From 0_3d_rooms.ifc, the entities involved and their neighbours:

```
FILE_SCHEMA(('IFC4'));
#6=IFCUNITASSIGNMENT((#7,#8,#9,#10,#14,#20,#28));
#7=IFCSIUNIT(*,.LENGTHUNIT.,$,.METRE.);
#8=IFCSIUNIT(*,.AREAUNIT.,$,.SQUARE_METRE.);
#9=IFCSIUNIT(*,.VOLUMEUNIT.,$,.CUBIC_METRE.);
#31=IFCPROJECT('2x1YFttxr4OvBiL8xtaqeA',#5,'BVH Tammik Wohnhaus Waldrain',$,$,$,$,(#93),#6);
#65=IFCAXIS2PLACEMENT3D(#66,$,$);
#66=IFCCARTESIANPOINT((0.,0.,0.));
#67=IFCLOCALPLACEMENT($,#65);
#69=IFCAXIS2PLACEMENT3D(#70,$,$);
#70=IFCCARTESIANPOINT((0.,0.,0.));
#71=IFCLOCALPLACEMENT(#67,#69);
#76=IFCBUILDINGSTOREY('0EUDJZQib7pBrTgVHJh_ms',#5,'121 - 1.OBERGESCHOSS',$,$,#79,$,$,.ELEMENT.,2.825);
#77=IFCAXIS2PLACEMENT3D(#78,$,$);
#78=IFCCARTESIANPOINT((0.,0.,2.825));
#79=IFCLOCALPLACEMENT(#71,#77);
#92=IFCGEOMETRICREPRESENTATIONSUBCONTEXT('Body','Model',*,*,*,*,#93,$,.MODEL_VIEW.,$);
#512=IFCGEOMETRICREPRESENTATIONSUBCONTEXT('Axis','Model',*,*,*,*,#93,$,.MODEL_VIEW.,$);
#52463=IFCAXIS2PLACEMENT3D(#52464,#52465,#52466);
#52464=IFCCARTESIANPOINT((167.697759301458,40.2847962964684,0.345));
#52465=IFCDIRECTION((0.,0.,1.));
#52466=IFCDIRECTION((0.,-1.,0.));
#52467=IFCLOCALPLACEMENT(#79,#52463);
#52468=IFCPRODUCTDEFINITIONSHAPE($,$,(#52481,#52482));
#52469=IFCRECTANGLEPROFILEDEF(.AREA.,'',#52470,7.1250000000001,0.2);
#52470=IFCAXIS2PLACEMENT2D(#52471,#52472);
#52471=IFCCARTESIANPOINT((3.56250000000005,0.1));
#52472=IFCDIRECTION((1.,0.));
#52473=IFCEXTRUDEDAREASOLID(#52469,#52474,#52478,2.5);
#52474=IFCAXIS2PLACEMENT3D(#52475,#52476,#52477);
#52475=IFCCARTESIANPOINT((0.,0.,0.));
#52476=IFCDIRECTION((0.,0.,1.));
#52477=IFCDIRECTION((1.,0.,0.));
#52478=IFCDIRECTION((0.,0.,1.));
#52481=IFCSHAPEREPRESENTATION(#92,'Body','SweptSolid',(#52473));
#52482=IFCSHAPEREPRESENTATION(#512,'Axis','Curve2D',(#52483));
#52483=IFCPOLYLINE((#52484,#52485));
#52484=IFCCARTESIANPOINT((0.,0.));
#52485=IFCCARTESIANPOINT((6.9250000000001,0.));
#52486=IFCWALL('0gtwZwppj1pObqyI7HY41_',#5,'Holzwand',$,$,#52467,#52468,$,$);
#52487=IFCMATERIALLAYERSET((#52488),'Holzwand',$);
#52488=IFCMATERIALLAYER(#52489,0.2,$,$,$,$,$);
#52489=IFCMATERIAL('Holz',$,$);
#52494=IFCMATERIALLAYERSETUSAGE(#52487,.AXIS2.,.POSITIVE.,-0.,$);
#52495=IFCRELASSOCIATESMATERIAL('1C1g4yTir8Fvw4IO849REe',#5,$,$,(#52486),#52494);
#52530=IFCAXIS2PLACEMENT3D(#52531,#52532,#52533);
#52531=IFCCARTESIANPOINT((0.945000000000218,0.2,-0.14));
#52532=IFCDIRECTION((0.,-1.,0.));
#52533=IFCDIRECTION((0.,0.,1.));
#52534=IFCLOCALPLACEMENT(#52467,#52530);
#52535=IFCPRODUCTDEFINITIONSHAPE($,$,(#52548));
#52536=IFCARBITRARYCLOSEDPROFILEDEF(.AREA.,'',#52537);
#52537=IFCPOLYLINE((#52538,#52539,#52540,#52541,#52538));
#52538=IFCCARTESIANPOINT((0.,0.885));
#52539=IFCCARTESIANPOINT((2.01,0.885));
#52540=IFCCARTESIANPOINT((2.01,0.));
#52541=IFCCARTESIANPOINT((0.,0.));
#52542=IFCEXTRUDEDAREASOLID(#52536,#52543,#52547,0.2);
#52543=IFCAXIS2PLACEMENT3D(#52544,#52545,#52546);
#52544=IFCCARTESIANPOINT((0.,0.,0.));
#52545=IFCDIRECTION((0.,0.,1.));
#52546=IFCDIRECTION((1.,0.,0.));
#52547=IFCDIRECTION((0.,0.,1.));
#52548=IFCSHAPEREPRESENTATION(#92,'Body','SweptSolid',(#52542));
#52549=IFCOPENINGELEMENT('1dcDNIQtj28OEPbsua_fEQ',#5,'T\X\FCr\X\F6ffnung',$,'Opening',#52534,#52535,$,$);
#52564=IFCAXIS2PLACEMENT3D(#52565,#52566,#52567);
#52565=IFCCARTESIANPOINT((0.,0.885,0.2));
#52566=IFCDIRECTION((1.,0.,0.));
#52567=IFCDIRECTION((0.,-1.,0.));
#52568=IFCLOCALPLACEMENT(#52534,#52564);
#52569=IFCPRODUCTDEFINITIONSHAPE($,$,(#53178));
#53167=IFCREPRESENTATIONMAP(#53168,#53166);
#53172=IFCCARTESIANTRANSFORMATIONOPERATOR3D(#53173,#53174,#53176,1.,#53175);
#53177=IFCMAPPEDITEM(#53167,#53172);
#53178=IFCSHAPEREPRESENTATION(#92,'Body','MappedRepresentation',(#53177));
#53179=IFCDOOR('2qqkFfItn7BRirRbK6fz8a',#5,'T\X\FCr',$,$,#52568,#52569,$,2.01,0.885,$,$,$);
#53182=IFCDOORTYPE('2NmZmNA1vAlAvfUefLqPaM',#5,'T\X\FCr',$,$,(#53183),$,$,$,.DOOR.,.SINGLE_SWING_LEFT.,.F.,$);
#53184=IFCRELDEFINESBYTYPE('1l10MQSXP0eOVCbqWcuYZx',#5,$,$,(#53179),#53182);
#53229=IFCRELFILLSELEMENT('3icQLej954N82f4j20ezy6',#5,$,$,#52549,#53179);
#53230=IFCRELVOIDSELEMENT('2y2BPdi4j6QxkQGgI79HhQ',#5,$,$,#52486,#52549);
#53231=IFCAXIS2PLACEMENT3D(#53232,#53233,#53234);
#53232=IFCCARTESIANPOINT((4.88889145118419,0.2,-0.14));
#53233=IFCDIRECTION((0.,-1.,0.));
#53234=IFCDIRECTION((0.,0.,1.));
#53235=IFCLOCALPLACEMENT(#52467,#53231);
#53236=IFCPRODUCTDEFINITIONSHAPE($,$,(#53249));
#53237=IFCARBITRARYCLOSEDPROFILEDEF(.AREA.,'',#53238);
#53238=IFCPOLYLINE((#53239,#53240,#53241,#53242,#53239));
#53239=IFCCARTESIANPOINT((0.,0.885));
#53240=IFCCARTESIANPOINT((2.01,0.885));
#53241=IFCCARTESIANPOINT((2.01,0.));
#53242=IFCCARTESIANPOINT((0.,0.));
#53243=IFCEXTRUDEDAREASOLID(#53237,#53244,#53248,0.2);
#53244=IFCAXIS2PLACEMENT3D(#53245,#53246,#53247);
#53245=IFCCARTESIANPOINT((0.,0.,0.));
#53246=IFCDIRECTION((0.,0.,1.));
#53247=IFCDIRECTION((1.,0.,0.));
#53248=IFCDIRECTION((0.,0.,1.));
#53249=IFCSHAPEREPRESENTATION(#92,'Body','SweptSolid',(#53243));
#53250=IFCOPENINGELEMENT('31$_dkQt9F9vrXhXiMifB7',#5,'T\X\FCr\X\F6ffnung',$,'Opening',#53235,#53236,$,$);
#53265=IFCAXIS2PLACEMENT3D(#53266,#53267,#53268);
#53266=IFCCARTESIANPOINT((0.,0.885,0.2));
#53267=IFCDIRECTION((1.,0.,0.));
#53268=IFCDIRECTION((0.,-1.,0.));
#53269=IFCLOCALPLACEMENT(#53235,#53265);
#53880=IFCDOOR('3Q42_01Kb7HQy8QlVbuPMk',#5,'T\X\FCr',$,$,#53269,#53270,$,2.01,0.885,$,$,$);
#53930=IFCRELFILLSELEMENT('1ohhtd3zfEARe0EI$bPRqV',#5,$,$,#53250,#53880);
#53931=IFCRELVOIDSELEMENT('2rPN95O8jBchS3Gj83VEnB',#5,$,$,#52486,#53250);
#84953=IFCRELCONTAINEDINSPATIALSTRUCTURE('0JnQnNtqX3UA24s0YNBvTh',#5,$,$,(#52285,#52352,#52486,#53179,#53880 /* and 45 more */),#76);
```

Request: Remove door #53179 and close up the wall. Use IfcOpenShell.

```python
import ifcopenshell
import ifcopenshell.api.feature
import ifcopenshell.api.root
import ifcopenshell.geom
import ifcopenshell.util.shape

model = ifcopenshell.open("0_3d_rooms.ifc")
settings = ifcopenshell.geom.settings()


def volume(element):
    """Net volume in cubic metres, openings subtracted."""
    shape = ifcopenshell.geom.create_shape(settings, element)
    return ifcopenshell.util.shape.get_volume(shape.geometry)


door = model.by_id(53179)
opening = door.FillsVoids[0].RelatingOpeningElement
wall = opening.VoidsElements[0].RelatingBuildingElement
before = volume(wall)

ifcopenshell.api.root.remove_product(model, product=door)
ifcopenshell.api.feature.remove_feature(model, feature=opening)

after = volume(wall)

print(f"wall volume {before:.3f} -> {after:.3f} m3")

model.write("0_3d_rooms_v2.ifc")
```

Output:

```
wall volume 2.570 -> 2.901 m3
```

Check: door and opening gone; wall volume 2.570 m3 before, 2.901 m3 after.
